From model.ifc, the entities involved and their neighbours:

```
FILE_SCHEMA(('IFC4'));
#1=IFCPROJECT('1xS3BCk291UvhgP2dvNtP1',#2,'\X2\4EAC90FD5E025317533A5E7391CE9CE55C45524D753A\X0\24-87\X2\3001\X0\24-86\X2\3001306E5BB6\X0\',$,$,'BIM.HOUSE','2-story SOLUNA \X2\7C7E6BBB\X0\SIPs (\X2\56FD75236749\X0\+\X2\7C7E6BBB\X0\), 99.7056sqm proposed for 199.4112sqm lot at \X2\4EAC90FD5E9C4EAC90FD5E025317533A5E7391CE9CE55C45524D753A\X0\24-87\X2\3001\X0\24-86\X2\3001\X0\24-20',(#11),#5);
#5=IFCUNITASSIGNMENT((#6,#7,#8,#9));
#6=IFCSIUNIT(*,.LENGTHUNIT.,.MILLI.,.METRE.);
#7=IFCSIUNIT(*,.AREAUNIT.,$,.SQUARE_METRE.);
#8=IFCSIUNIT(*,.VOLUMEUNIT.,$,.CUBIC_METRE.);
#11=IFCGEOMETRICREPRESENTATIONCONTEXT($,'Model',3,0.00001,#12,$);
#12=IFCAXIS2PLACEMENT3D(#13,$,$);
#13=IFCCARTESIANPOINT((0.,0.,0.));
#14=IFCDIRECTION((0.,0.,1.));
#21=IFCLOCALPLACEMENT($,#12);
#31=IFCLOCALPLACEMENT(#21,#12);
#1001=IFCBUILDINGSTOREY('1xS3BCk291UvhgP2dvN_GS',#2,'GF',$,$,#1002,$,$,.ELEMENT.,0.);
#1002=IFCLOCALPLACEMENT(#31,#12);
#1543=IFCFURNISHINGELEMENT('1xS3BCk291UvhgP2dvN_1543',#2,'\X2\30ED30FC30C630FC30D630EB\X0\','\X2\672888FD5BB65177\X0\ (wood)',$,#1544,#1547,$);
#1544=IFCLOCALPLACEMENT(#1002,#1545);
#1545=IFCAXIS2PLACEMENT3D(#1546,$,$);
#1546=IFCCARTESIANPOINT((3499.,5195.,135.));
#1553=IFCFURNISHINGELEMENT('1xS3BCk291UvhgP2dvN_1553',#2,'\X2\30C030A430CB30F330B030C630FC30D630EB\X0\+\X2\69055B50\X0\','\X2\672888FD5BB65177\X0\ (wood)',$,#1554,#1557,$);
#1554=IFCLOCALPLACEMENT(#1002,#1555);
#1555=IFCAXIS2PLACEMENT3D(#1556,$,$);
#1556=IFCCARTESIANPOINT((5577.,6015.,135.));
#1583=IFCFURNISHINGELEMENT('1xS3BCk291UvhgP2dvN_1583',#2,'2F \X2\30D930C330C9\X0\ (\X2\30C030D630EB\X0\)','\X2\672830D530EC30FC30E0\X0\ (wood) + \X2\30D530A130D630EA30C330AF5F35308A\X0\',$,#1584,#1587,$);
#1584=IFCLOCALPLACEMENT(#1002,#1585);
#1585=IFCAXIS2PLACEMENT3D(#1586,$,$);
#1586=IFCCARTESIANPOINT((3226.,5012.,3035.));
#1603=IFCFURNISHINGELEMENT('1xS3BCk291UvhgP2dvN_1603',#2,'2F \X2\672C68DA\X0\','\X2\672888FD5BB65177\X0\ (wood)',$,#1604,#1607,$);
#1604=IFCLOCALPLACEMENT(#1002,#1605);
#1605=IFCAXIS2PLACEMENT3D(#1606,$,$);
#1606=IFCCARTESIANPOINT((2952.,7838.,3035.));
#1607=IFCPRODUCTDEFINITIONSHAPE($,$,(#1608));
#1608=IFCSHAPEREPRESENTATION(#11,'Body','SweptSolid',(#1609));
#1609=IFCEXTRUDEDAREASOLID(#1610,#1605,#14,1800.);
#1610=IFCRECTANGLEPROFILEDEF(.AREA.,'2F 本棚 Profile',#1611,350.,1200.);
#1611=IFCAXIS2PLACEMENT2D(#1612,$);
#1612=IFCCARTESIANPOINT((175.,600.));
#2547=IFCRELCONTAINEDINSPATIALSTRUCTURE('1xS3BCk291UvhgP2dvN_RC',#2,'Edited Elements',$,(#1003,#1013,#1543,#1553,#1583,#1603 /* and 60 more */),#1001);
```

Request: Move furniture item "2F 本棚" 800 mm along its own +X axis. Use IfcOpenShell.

```python
import ifcopenshell
import ifcopenshell.api.geometry
import ifcopenshell.util.placement
import ifcopenshell.util.unit

model = ifcopenshell.open("model.ifc")
unit_scale = ifcopenshell.util.unit.calculate_unit_scale(model)

item = model.by_id(1603)
matrix = ifcopenshell.util.placement.get_local_placement(item.ObjectPlacement)
matrix[:3, 3] += matrix[:3, 0] * 0.8 / unit_scale
ifcopenshell.api.geometry.edit_object_placement(model, product=item, matrix=matrix, is_si=False)

print(ifcopenshell.util.placement.get_local_placement(item.ObjectPlacement).round(3) + 0.0)

model.write("model_rev.ifc")
```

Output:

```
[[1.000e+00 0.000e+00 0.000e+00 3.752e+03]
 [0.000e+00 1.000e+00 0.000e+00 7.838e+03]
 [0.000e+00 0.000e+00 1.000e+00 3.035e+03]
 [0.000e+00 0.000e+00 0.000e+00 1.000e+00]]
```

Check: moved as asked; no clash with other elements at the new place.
